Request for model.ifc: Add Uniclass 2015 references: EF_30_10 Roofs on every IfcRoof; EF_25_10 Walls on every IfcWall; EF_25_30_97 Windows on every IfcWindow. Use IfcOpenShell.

First a look at what the model holds.

```python
import ifcopenshell

model = ifcopenshell.open("model.ifc")
print(model.schema)
print("classifications:", [c.Name for c in model.by_type("IfcClassification")])
for ifc_class in ("IfcDoor", "IfcRoof", "IfcStair", "IfcWall", "IfcWindow"):
    print(ifc_class, len(model.by_type(ifc_class)))
```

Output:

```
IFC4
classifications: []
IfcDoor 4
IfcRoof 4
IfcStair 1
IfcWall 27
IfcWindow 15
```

```python
import ifcopenshell
import ifcopenshell.api.classification

model = ifcopenshell.open("model.ifc")

system = ifcopenshell.api.classification.add_classification(model, classification="Uniclass 2015")

codes = {
    "IfcRoof": ("EF_30_10", "Roofs"),
    "IfcWall": ("EF_25_10", "Walls"),
    "IfcWindow": ("EF_25_30_97", "Windows"),
}
for ifc_class, (code, name) in codes.items():
    products = model.by_type(ifc_class)
    ifcopenshell.api.classification.add_reference(
        model, products=products, classification=system, identification=code, name=name
    )
    print(code, len(products))

model.write("model_edited.ifc")
```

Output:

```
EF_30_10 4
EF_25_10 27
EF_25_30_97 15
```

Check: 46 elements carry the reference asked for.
